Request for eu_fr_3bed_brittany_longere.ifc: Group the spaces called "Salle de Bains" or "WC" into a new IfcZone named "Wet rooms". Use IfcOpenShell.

First a look at what the model holds.

```python
import ifcopenshell

model = ifcopenshell.open("eu_fr_3bed_brittany_longere.ifc")
print(model.schema)
seen = {}
for space in model.by_type("IfcSpace"):
    seen[space.LongName] = seen.get(space.LongName, 0) + 1
for name, count in sorted(seen.items(), key=str):
    print(count, "x", name)
print("zones:", [z.Name for z in model.by_type("IfcZone")][:20])
```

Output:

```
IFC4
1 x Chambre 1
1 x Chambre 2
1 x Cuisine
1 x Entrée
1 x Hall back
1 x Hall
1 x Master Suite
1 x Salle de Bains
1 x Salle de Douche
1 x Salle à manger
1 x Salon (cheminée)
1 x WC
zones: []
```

```python
import ifcopenshell
import ifcopenshell.api.group
import ifcopenshell.api.root

model = ifcopenshell.open("eu_fr_3bed_brittany_longere.ifc")

names = {"Salle de Bains", "WC"}
spaces = [s for s in model.by_type("IfcSpace") if s.LongName in names]

zone = ifcopenshell.api.root.create_entity(model, ifc_class="IfcZone", name="Wet rooms")
ifcopenshell.api.group.assign_group(model, products=spaces, group=zone)
print(len(spaces), "spaces in", zone.Name)

model.write("eu_fr_3bed_brittany_longere-out.ifc")
```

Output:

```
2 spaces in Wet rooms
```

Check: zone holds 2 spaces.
